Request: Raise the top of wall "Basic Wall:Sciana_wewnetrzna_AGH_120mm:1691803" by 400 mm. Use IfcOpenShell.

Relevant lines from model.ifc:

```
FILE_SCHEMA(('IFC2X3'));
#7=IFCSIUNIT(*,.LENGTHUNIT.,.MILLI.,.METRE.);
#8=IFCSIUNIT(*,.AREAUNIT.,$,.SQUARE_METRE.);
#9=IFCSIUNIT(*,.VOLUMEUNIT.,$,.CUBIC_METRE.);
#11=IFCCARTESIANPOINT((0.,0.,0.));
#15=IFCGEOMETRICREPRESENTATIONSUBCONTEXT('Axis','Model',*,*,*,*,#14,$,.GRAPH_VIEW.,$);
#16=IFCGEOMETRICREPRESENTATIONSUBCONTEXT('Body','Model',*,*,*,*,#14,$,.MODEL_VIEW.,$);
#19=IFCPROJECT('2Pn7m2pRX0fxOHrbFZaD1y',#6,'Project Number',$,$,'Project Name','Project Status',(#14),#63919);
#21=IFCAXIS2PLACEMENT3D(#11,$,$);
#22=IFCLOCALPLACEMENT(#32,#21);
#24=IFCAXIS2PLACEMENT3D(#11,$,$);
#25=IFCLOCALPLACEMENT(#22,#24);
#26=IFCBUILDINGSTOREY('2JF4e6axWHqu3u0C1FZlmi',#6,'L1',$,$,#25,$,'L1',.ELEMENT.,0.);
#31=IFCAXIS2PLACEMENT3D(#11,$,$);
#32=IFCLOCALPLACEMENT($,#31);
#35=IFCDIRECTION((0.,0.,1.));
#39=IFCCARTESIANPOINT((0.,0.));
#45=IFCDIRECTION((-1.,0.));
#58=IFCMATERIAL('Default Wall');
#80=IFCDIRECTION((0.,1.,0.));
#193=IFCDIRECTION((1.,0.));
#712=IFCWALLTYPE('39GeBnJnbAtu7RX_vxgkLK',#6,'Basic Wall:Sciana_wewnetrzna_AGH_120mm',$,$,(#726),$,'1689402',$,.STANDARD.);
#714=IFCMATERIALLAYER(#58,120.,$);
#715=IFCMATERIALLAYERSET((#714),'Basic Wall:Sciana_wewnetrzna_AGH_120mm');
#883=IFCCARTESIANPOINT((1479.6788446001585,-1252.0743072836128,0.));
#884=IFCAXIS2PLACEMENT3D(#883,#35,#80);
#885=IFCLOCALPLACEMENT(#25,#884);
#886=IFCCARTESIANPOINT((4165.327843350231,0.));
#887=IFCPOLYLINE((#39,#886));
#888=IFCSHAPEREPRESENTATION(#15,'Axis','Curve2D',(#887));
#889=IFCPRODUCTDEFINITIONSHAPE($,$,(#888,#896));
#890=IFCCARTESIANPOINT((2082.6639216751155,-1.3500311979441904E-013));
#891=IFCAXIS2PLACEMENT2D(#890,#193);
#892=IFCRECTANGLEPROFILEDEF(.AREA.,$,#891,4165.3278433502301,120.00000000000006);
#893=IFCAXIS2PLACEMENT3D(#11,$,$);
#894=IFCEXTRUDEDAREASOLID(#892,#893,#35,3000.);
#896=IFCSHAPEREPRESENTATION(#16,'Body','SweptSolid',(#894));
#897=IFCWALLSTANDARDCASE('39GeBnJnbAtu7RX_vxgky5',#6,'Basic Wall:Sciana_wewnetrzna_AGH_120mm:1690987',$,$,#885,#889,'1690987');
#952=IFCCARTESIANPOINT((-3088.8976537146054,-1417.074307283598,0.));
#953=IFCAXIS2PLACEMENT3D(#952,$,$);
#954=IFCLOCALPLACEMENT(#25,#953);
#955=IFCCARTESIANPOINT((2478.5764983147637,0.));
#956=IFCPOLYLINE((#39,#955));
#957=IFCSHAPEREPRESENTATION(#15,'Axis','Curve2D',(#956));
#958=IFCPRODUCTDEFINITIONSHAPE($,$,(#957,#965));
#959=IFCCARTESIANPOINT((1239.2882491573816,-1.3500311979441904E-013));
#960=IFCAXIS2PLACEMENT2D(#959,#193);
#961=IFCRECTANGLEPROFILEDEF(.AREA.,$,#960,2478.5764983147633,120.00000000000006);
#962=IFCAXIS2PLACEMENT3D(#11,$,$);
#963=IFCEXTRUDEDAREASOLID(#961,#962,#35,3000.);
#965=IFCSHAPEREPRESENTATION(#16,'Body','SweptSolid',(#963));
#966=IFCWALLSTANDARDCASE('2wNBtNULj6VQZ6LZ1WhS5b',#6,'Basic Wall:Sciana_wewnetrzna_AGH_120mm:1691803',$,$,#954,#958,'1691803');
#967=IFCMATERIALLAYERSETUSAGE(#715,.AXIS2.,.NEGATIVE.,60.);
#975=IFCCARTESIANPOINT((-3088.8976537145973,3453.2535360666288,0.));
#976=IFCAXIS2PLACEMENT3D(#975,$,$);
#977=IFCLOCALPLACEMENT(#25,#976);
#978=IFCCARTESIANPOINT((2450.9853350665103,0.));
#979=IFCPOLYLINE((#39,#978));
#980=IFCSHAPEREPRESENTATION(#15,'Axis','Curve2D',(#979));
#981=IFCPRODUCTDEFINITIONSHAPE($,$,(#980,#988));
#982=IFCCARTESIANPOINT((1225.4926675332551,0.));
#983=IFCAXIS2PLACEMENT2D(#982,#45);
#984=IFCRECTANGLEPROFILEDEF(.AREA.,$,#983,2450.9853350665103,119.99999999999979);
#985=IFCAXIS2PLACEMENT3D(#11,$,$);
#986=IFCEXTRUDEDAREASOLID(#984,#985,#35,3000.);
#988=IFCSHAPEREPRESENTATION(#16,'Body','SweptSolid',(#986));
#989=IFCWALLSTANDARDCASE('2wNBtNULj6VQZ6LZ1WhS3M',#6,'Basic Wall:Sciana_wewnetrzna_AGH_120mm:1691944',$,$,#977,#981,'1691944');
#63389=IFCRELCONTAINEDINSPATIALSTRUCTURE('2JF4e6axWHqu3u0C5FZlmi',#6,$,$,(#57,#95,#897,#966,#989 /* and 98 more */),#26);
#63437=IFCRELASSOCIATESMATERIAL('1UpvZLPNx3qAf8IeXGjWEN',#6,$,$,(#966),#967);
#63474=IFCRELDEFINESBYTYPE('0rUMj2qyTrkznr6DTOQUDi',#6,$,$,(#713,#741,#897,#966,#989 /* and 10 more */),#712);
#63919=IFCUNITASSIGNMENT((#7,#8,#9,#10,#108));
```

```python
import ifcopenshell
import ifcopenshell.geom
import ifcopenshell.util.representation
import ifcopenshell.util.shape

model = ifcopenshell.open("model.ifc")
settings = ifcopenshell.geom.settings()


def volume(element):
    """Net volume in cubic metres, openings subtracted."""
    shape = ifcopenshell.geom.create_shape(settings, element)
    return ifcopenshell.util.shape.get_volume(shape.geometry)


wall = model.by_guid("2wNBtNULj6VQZ6LZ1WhS5b")
before = volume(wall)

body = ifcopenshell.util.representation.get_representation(wall, "Model", "Body")
solid = body.Items[0]
old_height = solid.Depth
solid.Depth += 400.0
after = volume(wall)

print(f"height {old_height:g} -> {solid.Depth:g}, volume {before:.3f} -> {after:.3f} m3")

model.write("model_rev.ifc")
```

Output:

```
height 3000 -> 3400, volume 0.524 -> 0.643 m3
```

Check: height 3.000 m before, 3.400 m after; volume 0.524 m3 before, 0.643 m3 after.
